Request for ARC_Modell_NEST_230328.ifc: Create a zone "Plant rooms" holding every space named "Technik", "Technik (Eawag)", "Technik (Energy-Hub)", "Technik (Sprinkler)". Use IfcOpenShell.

First a look at what the model holds.

```python
import ifcopenshell

model = ifcopenshell.open("ARC_Modell_NEST_230328.ifc")
print(model.schema)
seen = {}
for space in model.by_type("IfcSpace"):
    seen[space.LongName] = seen.get(space.LongName, 0) + 1
for name, count in sorted(seen.items(), key=str):
    print(count, "x", name)
print("zones:", [z.Name for z in model.by_type("IfcZone")][:20])
```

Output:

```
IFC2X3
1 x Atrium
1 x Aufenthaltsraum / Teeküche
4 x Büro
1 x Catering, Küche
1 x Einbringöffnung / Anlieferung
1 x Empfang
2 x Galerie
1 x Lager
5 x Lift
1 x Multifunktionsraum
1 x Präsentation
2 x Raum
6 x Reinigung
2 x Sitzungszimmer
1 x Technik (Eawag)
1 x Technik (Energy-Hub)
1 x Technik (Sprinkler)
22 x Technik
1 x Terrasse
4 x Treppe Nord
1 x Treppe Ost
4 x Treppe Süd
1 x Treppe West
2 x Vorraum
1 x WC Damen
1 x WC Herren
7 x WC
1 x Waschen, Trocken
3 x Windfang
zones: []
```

```python
import ifcopenshell
import ifcopenshell.api.group
import ifcopenshell.api.root

model = ifcopenshell.open("ARC_Modell_NEST_230328.ifc")

names = {"Technik", "Technik (Eawag)", "Technik (Energy-Hub)", "Technik (Sprinkler)"}
spaces = [s for s in model.by_type("IfcSpace") if s.LongName in names]

zone = ifcopenshell.api.root.create_entity(model, ifc_class="IfcZone", name="Plant rooms")
ifcopenshell.api.group.assign_group(model, products=spaces, group=zone)
print(len(spaces), "spaces in", zone.Name)

model.write("ARC_Modell_NEST_230328_updated.ifc")
```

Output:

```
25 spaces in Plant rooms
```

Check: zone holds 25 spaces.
